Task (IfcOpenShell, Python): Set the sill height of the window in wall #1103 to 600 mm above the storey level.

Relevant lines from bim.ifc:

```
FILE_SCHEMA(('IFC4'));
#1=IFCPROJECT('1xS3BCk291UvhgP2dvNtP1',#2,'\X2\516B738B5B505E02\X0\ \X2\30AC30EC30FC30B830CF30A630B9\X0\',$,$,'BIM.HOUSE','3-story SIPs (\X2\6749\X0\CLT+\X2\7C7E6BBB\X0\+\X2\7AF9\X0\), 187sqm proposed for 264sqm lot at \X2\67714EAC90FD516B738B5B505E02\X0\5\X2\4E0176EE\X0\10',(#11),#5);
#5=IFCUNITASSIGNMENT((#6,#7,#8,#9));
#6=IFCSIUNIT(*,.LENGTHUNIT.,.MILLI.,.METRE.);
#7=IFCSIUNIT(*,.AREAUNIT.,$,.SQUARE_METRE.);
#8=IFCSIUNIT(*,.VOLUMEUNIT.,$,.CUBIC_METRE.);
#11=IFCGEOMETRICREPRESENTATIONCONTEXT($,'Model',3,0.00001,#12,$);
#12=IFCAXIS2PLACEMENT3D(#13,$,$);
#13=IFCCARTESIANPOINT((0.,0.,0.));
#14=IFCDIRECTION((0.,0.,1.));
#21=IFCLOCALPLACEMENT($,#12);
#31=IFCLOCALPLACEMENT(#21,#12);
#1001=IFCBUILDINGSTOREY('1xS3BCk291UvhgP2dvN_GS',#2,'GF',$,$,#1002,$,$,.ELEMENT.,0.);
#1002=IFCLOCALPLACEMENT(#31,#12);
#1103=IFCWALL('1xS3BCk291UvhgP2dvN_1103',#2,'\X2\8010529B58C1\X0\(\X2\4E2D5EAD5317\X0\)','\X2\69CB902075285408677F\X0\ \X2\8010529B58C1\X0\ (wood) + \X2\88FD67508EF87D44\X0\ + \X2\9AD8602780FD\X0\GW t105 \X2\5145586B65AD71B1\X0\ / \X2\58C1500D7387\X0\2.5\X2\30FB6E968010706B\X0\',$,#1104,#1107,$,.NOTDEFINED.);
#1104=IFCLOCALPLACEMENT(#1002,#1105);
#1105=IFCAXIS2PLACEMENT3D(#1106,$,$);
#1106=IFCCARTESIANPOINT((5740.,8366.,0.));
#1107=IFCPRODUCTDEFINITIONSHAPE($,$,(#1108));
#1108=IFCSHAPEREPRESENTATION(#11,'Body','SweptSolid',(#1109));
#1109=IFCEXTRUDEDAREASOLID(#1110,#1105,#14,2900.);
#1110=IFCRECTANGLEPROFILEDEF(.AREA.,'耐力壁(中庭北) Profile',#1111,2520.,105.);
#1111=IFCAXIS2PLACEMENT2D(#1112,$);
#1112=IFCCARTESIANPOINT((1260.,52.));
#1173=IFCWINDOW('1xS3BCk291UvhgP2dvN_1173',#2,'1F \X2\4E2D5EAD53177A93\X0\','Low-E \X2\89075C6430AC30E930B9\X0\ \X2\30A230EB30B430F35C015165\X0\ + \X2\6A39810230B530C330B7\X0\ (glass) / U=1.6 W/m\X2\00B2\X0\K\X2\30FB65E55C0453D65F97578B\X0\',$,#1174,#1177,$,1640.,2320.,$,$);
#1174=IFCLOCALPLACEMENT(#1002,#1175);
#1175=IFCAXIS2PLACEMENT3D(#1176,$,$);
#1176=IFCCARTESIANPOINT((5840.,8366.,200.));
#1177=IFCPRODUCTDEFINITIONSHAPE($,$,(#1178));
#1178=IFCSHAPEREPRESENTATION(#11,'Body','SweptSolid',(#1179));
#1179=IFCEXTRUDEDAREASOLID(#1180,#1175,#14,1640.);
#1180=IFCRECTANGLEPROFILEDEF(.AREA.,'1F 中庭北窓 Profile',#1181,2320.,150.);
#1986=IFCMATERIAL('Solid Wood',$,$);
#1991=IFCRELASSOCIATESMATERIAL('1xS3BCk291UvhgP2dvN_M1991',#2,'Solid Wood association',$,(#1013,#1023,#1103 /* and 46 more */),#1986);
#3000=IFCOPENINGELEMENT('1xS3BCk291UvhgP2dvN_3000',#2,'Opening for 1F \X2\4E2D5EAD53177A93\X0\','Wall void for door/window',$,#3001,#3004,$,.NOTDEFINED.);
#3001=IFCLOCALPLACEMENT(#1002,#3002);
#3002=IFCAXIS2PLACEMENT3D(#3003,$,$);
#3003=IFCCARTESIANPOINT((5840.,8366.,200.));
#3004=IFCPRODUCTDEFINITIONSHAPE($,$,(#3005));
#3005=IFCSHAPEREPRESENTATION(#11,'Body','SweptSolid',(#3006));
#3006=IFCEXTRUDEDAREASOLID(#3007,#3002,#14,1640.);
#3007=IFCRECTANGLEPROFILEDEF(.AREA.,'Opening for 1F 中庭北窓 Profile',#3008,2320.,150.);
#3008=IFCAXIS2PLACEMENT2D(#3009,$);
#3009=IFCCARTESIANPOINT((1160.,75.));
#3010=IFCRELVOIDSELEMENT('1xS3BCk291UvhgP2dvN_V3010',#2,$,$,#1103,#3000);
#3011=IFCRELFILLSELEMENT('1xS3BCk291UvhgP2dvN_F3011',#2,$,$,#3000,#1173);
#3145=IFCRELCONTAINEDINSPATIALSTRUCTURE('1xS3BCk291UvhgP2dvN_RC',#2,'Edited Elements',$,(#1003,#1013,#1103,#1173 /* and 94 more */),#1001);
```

```python
import numpy as np
import ifcopenshell
import ifcopenshell.api.geometry
import ifcopenshell.geom
import ifcopenshell.util.element
import ifcopenshell.util.placement
import ifcopenshell.util.shape
import ifcopenshell.util.unit

model = ifcopenshell.open("bim.ifc")
unit_scale = ifcopenshell.util.unit.calculate_unit_scale(model)

window = model.by_guid("1xS3BCk291UvhgP2dvN_1173")
opening = window.FillsVoids[0].RelatingOpeningElement
storey = ifcopenshell.util.element.get_container(window, ifc_class="IfcBuildingStorey")
level = ifcopenshell.util.placement.get_local_placement(storey.ObjectPlacement)[2, 3]

# The opening's origin need not be at the sill, so measure its lowest point.
shape = ifcopenshell.geom.create_shape(ifcopenshell.geom.settings(), opening)
bottom = ifcopenshell.util.shape.get_shape_bottom_elevation(shape, shape.geometry) / unit_scale
dz = level + 600.0 - bottom

shift = np.array([0.0, 0.0, dz])
# The window is not placed relative to its opening, so move both.
for product in (opening, window):
    matrix = ifcopenshell.util.placement.get_local_placement(product.ObjectPlacement)
    matrix[:3, 3] += shift
    ifcopenshell.api.geometry.edit_object_placement(model, product=product, matrix=matrix, is_si=False)

print(f"moved by {dz * unit_scale:+.3f} m")

model.write("bim-out.ifc")
```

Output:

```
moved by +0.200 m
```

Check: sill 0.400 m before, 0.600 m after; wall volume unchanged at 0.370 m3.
